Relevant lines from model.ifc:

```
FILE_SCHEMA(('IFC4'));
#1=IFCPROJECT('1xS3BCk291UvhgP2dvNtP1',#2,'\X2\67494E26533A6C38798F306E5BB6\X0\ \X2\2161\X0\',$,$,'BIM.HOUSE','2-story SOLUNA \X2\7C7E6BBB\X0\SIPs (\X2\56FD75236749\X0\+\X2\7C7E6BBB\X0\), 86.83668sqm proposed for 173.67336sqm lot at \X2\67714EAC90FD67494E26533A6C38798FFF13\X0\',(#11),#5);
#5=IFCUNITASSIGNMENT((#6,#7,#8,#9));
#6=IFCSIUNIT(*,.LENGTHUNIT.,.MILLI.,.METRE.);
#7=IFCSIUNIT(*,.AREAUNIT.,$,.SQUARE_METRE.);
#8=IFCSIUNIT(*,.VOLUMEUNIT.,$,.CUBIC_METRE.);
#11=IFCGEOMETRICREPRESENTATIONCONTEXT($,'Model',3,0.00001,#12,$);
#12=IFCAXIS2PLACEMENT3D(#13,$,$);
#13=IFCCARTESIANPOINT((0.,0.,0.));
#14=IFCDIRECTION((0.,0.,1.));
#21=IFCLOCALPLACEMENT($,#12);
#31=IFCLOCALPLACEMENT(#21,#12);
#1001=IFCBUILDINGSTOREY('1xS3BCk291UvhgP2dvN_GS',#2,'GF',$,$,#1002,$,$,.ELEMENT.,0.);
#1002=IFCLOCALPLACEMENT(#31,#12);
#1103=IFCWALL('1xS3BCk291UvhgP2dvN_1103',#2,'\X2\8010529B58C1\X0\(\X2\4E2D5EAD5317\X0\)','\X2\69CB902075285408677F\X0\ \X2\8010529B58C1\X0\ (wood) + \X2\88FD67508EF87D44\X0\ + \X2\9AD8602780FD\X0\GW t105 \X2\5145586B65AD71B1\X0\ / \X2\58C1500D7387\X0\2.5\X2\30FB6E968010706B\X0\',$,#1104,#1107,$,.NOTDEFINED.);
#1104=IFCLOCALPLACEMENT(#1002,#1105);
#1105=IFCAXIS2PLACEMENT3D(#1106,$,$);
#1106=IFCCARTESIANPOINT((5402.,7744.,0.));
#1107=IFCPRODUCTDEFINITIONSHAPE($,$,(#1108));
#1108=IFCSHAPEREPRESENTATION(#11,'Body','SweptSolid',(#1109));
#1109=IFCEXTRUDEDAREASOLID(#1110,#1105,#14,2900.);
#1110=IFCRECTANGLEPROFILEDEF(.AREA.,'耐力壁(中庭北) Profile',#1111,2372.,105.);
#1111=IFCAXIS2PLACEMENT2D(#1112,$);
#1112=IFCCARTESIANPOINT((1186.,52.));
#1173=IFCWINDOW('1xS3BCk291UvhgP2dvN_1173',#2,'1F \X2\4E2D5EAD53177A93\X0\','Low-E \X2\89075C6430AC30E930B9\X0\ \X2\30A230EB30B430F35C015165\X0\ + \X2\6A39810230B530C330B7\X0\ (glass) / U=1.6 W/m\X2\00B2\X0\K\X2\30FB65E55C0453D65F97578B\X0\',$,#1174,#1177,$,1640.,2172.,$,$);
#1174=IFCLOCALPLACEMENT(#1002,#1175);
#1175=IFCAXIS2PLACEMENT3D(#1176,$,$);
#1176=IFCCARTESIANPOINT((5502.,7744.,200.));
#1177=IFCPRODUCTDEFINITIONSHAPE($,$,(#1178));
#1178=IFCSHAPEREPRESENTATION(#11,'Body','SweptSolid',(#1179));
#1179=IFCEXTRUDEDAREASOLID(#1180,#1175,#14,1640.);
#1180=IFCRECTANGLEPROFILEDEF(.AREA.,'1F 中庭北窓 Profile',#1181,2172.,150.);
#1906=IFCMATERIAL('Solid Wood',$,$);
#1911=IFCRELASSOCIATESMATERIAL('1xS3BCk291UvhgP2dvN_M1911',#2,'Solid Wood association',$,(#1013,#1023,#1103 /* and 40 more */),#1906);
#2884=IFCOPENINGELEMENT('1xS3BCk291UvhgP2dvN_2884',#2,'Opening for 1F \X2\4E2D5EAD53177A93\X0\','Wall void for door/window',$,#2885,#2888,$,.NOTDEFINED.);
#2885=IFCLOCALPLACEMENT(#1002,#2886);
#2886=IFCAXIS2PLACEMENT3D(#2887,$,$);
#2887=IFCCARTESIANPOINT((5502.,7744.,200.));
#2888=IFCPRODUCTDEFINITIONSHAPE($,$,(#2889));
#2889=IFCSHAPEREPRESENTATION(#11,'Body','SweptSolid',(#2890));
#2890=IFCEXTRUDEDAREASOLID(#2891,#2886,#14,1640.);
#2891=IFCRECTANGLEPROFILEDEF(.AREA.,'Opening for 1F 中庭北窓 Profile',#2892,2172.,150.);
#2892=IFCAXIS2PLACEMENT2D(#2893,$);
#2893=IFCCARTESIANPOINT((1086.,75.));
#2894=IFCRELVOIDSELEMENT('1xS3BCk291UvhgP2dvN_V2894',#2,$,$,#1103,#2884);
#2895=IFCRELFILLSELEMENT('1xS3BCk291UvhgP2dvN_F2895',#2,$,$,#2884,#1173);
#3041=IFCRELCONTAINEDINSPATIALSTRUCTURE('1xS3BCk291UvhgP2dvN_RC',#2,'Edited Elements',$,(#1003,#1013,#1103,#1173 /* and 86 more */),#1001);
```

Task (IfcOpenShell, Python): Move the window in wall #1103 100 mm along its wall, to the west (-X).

```python
import ifcopenshell
import ifcopenshell.api.geometry
import ifcopenshell.util.placement
import ifcopenshell.util.unit

model = ifcopenshell.open("model.ifc")
unit_scale = ifcopenshell.util.unit.calculate_unit_scale(model)

window = model.by_guid("1xS3BCk291UvhgP2dvN_1173")
opening = window.FillsVoids[0].RelatingOpeningElement
wall = opening.VoidsElements[0].RelatingBuildingElement

wall_matrix = ifcopenshell.util.placement.get_local_placement(wall.ObjectPlacement)
shift = wall_matrix[:3, 0] * -0.1 / unit_scale
before = ifcopenshell.util.placement.get_local_placement(window.ObjectPlacement)[:3, 3].copy()

# The window is not placed relative to its opening, so move both.
for product in (opening, window):
    matrix = ifcopenshell.util.placement.get_local_placement(product.ObjectPlacement)
    matrix[:3, 3] += shift
    ifcopenshell.api.geometry.edit_object_placement(model, product=product, matrix=matrix, is_si=False)

after = ifcopenshell.util.placement.get_local_placement(window.ObjectPlacement)[:3, 3]
print("window moved by", (after - before).round(3) + 0.0)

model.write("model_edited.ifc")
```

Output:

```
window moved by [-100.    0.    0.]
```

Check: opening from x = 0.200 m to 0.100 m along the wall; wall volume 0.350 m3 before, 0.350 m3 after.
